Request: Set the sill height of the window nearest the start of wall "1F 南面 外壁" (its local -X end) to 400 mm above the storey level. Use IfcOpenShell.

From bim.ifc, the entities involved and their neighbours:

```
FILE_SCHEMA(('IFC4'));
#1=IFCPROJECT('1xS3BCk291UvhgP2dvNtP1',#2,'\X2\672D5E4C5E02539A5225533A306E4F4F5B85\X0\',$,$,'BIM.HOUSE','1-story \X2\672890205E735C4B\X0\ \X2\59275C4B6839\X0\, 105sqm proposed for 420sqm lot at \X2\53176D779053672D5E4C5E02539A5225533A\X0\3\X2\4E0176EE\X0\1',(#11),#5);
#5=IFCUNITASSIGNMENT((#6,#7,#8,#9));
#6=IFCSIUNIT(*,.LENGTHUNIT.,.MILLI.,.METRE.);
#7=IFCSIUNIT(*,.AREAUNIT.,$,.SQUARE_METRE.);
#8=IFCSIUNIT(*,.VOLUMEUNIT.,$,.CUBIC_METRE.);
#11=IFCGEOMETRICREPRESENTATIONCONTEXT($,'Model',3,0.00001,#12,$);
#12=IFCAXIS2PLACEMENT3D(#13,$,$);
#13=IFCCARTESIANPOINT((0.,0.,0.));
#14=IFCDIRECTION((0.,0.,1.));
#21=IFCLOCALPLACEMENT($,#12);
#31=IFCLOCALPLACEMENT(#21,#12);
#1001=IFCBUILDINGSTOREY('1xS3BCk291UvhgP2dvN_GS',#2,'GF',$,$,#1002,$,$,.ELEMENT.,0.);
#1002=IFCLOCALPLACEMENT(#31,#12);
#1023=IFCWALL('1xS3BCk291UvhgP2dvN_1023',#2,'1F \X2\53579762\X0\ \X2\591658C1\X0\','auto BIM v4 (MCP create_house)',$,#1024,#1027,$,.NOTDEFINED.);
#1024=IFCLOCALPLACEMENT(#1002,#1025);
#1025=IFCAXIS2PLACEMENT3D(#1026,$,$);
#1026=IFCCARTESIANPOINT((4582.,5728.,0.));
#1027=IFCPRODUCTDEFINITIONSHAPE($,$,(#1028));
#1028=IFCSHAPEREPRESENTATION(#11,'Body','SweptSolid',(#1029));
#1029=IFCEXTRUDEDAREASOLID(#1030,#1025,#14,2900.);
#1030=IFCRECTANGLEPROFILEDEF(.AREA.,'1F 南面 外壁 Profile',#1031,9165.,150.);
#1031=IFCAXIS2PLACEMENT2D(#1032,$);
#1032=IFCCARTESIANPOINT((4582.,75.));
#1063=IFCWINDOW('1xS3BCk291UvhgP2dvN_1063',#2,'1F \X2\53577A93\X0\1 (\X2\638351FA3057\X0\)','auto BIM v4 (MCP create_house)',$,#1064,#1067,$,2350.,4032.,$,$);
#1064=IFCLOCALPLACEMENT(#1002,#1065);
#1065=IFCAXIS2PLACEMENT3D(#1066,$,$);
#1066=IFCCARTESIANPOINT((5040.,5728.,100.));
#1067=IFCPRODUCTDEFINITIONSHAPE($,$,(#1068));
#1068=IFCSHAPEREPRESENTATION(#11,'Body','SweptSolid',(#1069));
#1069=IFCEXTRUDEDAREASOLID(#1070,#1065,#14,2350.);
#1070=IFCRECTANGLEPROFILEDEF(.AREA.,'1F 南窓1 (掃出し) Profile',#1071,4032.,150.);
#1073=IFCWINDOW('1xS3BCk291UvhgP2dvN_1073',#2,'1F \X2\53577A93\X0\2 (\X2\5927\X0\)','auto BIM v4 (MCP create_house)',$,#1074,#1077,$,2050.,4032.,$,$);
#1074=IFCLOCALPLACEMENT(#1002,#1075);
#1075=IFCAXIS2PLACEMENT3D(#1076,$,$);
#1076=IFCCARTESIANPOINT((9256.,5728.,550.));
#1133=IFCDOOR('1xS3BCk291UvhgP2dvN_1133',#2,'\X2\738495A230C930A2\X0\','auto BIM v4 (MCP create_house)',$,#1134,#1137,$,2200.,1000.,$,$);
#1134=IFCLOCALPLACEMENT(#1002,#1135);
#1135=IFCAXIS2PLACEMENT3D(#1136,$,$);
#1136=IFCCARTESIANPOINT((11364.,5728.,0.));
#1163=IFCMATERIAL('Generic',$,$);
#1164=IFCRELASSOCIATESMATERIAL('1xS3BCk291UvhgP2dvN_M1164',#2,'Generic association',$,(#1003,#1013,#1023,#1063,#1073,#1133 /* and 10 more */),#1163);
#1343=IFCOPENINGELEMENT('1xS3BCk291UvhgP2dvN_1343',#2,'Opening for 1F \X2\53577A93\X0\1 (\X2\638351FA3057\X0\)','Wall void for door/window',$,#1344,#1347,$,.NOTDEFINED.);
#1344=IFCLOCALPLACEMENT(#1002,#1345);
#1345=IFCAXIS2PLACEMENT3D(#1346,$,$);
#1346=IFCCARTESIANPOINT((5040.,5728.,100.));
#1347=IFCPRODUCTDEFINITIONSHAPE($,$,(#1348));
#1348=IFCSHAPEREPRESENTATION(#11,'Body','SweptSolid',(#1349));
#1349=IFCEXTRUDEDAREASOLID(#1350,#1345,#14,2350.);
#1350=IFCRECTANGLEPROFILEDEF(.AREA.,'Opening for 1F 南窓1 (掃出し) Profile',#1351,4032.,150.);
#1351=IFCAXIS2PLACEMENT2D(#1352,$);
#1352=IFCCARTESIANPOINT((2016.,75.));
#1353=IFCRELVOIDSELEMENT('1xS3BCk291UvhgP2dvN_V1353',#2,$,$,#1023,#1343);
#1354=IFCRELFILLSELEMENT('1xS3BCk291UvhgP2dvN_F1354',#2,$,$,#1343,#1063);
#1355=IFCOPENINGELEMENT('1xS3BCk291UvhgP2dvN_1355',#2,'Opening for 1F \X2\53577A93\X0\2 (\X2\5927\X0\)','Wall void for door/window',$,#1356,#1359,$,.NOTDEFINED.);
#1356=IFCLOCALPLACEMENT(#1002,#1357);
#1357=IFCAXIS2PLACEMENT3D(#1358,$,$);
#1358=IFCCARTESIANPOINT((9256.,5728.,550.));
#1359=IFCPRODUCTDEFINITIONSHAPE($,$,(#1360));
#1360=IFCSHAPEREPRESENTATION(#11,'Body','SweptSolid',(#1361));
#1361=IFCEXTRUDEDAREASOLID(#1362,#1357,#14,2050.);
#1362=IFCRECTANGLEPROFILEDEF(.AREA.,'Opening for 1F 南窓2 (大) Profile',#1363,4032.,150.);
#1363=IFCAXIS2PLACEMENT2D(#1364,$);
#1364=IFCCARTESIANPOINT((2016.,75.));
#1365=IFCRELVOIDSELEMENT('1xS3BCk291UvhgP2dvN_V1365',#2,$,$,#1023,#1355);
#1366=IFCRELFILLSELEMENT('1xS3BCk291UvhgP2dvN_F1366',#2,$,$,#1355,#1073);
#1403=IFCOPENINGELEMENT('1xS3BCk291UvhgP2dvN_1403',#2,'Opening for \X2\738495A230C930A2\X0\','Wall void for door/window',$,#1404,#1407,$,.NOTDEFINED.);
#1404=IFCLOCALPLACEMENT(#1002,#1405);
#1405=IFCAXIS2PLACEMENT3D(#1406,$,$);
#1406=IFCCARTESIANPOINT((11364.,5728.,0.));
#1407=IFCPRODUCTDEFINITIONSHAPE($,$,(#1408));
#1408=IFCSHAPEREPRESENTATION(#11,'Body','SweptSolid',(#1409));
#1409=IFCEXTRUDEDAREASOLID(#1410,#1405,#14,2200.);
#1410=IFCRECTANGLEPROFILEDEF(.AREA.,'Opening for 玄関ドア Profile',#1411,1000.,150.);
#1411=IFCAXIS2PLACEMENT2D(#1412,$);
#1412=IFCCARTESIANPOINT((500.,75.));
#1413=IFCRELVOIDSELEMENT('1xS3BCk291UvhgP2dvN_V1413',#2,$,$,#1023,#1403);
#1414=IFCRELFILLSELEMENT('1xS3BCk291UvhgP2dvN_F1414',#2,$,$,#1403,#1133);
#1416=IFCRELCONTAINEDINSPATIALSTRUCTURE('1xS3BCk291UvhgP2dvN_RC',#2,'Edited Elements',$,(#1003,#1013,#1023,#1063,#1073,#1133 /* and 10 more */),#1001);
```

```python
import numpy as np
import ifcopenshell
import ifcopenshell.api.geometry
import ifcopenshell.geom
import ifcopenshell.util.element
import ifcopenshell.util.placement
import ifcopenshell.util.shape
import ifcopenshell.util.unit

model = ifcopenshell.open("bim.ifc")
unit_scale = ifcopenshell.util.unit.calculate_unit_scale(model)

window = model.by_id(1063)
opening = window.FillsVoids[0].RelatingOpeningElement
storey = ifcopenshell.util.element.get_container(window, ifc_class="IfcBuildingStorey")
level = ifcopenshell.util.placement.get_local_placement(storey.ObjectPlacement)[2, 3]

# The opening's origin need not be at the sill, so measure its lowest point.
shape = ifcopenshell.geom.create_shape(ifcopenshell.geom.settings(), opening)
bottom = ifcopenshell.util.shape.get_shape_bottom_elevation(shape, shape.geometry) / unit_scale
dz = level + 0.4 / unit_scale - bottom

shift = np.array([0.0, 0.0, dz])
# The window is not placed relative to its opening, so move both.
for product in (opening, window):
    matrix = ifcopenshell.util.placement.get_local_placement(product.ObjectPlacement)
    matrix[:3, 3] += shift
    ifcopenshell.api.geometry.edit_object_placement(model, product=product, matrix=matrix, is_si=False)

print(f"moved by {dz * unit_scale:+.3f} m")

model.write("bim-out.ifc")
```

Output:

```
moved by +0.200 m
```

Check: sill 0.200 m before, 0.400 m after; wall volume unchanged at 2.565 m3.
